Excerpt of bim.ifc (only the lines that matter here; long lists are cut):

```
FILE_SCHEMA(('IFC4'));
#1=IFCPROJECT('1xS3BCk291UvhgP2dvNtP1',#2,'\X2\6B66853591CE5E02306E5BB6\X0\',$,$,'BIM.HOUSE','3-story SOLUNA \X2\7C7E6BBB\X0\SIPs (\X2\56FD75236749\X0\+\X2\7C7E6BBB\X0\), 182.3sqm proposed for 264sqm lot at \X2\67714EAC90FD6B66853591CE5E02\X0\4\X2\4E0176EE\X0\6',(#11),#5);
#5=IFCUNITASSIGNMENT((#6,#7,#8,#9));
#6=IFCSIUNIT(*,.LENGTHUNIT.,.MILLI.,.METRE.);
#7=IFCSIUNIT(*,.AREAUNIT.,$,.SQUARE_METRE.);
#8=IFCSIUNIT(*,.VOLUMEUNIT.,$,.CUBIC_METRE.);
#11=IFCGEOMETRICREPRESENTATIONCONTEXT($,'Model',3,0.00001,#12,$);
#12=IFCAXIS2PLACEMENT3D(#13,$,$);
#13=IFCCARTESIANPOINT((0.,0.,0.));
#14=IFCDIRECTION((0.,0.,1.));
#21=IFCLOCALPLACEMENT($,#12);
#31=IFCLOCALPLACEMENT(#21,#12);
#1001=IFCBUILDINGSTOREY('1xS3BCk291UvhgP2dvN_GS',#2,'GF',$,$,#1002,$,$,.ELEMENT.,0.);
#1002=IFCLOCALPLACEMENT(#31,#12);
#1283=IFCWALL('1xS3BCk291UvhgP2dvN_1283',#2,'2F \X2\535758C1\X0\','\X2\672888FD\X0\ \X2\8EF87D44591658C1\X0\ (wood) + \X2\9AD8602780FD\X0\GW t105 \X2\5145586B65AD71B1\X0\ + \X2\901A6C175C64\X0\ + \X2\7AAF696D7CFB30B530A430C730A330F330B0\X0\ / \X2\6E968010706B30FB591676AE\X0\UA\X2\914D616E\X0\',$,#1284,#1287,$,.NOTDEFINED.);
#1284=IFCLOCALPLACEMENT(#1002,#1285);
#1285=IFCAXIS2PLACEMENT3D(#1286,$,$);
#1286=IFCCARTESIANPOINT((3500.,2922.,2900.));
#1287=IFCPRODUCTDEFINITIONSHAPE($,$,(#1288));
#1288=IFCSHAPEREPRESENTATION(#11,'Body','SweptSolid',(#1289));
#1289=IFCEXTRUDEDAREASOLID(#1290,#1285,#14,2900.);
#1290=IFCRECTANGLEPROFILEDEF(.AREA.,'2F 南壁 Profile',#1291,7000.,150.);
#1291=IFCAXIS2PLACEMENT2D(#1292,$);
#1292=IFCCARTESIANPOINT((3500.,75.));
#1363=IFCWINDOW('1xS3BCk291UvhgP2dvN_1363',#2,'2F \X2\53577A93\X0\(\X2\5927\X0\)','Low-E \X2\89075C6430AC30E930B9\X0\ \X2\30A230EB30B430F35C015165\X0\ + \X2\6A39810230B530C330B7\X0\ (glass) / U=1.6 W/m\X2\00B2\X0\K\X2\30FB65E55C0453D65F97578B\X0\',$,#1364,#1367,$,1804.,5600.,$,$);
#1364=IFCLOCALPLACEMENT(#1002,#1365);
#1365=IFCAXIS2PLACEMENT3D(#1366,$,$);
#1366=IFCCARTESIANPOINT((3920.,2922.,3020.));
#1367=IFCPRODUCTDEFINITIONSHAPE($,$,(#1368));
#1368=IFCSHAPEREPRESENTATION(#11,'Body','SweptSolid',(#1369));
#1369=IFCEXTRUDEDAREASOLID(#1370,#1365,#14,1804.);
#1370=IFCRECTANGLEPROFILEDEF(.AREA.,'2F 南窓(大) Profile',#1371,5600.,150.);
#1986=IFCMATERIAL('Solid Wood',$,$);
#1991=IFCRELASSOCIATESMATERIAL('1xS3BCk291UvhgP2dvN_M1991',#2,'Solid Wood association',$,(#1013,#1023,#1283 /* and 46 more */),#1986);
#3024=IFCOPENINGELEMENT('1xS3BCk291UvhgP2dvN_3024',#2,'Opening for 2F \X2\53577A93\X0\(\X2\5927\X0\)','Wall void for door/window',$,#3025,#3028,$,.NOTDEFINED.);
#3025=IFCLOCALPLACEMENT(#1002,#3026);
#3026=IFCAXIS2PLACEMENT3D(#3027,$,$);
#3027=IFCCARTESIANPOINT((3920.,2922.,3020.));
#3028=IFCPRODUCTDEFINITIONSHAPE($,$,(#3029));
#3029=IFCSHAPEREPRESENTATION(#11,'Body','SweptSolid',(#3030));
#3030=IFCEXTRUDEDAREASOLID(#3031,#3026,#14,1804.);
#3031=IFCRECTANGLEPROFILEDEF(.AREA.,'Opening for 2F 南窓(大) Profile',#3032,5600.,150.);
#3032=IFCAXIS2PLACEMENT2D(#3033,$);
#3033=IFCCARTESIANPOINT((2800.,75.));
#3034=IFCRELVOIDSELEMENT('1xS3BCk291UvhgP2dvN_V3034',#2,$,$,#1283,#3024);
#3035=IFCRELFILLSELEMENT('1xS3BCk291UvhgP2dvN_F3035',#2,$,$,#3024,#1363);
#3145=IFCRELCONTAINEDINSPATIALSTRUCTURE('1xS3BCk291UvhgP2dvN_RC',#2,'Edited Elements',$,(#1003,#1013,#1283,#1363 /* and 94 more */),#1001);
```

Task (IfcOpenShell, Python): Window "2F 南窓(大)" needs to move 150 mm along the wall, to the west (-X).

```python
import ifcopenshell
import ifcopenshell.api.geometry
import ifcopenshell.util.placement

model = ifcopenshell.open("bim.ifc")

window = model.by_guid("1xS3BCk291UvhgP2dvN_1363")
opening = window.FillsVoids[0].RelatingOpeningElement
wall = opening.VoidsElements[0].RelatingBuildingElement

wall_matrix = ifcopenshell.util.placement.get_local_placement(wall.ObjectPlacement)
shift = wall_matrix[:3, 0] * -150.0
before = ifcopenshell.util.placement.get_local_placement(window.ObjectPlacement)[:3, 3].copy()

# The window is not placed relative to its opening, so move both.
for product in (opening, window):
    matrix = ifcopenshell.util.placement.get_local_placement(product.ObjectPlacement)
    matrix[:3, 3] += shift
    ifcopenshell.api.geometry.edit_object_placement(model, product=product, matrix=matrix, is_si=False)

after = ifcopenshell.util.placement.get_local_placement(window.ObjectPlacement)[:3, 3]
print("window moved by", (after - before).round(3) + 0.0)

model.write("bim-out.ifc")
```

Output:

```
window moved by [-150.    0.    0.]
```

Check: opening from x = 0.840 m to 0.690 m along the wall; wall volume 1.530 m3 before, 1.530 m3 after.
